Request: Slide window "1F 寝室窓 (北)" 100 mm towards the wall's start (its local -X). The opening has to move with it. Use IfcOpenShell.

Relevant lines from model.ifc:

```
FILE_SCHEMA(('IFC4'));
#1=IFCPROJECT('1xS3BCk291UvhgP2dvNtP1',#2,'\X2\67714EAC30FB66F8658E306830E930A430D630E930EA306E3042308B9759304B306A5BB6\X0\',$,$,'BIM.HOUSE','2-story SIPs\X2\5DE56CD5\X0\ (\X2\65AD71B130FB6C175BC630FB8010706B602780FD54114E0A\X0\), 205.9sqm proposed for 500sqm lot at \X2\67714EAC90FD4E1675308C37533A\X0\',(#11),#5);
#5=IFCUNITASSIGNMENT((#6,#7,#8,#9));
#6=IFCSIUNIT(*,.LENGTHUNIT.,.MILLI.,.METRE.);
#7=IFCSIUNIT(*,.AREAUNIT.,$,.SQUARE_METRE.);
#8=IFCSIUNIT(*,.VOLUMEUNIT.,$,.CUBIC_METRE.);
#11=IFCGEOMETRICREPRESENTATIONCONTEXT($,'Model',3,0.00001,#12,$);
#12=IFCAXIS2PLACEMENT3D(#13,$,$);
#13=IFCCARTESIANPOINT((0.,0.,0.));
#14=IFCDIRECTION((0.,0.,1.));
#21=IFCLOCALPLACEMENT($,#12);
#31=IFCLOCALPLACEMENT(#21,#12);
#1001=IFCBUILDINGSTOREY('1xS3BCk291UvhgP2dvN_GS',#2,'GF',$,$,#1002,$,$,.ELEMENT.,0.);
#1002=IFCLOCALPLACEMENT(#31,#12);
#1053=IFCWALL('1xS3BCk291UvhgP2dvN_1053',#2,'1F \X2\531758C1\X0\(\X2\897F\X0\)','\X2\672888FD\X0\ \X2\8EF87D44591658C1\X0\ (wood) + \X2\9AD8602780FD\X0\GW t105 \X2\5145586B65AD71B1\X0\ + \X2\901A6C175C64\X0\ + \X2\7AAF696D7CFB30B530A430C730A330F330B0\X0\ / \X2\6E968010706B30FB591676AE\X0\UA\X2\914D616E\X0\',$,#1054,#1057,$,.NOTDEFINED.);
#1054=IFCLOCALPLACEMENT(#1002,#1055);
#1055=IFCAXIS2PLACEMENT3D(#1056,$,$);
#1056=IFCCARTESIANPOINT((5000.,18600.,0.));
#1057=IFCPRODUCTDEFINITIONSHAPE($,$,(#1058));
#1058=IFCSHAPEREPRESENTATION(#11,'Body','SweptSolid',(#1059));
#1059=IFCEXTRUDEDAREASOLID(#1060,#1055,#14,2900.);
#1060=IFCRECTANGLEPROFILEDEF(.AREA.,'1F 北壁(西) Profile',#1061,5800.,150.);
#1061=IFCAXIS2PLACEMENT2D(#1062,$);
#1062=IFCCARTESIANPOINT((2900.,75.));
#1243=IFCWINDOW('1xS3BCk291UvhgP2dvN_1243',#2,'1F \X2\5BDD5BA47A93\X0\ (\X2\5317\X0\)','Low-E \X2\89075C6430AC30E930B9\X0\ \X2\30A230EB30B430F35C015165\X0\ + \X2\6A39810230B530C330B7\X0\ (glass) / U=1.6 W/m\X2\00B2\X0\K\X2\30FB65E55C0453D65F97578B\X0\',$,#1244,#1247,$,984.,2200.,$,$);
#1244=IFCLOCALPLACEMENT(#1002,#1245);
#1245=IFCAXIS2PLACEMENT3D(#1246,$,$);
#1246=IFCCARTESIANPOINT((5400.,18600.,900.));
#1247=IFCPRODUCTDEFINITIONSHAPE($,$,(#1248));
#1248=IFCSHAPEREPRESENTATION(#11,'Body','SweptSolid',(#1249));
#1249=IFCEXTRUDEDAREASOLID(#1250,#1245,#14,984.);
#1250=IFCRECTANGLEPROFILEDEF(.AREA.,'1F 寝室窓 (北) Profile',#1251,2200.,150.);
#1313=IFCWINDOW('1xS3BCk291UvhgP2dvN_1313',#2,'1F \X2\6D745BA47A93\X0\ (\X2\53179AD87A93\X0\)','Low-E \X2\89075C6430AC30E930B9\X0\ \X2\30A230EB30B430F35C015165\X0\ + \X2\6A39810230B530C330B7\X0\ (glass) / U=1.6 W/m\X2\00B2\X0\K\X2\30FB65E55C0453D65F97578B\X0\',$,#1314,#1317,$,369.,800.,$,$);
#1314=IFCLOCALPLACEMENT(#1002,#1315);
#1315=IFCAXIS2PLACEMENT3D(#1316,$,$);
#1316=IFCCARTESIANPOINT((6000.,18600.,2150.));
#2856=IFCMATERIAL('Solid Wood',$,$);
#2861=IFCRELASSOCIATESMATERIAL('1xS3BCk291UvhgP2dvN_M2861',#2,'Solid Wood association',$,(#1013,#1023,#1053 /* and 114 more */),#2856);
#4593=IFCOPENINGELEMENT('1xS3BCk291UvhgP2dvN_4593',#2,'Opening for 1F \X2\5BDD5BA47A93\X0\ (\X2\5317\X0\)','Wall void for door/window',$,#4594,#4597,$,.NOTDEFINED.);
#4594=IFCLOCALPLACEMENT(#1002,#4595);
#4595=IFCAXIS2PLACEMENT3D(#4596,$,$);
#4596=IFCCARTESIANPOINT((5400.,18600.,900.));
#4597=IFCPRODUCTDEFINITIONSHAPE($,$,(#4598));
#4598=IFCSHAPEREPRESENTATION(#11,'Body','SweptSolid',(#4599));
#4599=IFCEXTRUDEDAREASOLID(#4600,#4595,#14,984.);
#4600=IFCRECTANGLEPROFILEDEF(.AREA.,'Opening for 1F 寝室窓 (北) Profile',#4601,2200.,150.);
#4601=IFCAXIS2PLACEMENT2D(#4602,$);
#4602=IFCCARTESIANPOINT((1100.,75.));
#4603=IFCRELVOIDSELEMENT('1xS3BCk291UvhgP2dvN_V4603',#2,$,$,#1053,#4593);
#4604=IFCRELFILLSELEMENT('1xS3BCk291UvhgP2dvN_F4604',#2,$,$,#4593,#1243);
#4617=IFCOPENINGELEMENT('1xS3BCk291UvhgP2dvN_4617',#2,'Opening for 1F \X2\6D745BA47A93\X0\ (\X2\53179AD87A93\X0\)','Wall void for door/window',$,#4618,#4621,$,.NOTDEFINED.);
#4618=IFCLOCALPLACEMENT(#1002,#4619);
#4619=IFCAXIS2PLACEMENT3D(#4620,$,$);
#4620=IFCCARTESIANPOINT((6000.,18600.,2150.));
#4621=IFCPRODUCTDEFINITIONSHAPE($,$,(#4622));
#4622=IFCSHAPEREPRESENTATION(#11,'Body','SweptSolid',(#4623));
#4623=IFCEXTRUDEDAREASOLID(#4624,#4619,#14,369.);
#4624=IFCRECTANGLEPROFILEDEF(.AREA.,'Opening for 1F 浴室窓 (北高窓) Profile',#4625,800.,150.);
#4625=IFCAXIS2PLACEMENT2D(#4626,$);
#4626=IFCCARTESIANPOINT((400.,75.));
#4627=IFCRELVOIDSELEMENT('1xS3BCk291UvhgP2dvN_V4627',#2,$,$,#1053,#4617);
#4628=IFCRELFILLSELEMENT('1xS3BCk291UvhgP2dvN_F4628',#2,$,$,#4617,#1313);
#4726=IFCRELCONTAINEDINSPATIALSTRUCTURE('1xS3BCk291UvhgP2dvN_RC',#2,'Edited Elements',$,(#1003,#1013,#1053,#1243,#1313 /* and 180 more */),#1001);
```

```python
import ifcopenshell
import ifcopenshell.api.geometry
import ifcopenshell.util.placement
import ifcopenshell.util.unit

model = ifcopenshell.open("model.ifc")
unit_scale = ifcopenshell.util.unit.calculate_unit_scale(model)

window = model.by_guid("1xS3BCk291UvhgP2dvN_1243")
opening = window.FillsVoids[0].RelatingOpeningElement
wall = opening.VoidsElements[0].RelatingBuildingElement

wall_matrix = ifcopenshell.util.placement.get_local_placement(wall.ObjectPlacement)
shift = wall_matrix[:3, 0] * -0.1 / unit_scale
before = ifcopenshell.util.placement.get_local_placement(window.ObjectPlacement)[:3, 3].copy()

# The window is not placed relative to its opening, so move both.
for product in (opening, window):
    matrix = ifcopenshell.util.placement.get_local_placement(product.ObjectPlacement)
    matrix[:3, 3] += shift
    ifcopenshell.api.geometry.edit_object_placement(model, product=product, matrix=matrix, is_si=False)

after = ifcopenshell.util.placement.get_local_placement(window.ObjectPlacement)[:3, 3]
print("window moved by", (after - before).round(3) + 0.0)

model.write("model_v2.ifc")
```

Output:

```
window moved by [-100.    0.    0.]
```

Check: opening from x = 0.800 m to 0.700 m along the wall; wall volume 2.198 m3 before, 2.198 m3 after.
